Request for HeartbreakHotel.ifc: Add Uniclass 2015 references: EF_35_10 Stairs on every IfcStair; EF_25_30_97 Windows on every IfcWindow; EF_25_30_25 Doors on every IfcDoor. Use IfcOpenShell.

First a look at what the model holds.

```python
import ifcopenshell

model = ifcopenshell.open("HeartbreakHotel.ifc")
print(model.schema)
print("classifications:", [c.Name for c in model.by_type("IfcClassification")])
for ifc_class in ("IfcDoor", "IfcRoof", "IfcStair", "IfcWall", "IfcWindow"):
    print(ifc_class, len(model.by_type(ifc_class)))
```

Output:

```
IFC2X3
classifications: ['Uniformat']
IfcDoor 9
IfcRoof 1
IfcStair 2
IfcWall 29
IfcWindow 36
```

```python
import ifcopenshell
import ifcopenshell.api.classification

model = ifcopenshell.open("HeartbreakHotel.ifc")

# IFC2X3 requires Source and Edition and has no link from the project to the system.
system = model.create_entity("IfcClassification", Source="NBS", Edition="2015", Name="Uniclass 2015")

codes = {
    "IfcStair": ("EF_35_10", "Stairs"),
    "IfcWindow": ("EF_25_30_97", "Windows"),
    "IfcDoor": ("EF_25_30_25", "Doors"),
}
for ifc_class, (code, name) in codes.items():
    products = model.by_type(ifc_class)
    ifcopenshell.api.classification.add_reference(
        model, products=products, classification=system, identification=code, name=name
    )
    print(code, len(products))

model.write("HeartbreakHotel_v2.ifc")
```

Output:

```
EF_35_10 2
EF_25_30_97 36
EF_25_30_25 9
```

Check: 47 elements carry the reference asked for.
